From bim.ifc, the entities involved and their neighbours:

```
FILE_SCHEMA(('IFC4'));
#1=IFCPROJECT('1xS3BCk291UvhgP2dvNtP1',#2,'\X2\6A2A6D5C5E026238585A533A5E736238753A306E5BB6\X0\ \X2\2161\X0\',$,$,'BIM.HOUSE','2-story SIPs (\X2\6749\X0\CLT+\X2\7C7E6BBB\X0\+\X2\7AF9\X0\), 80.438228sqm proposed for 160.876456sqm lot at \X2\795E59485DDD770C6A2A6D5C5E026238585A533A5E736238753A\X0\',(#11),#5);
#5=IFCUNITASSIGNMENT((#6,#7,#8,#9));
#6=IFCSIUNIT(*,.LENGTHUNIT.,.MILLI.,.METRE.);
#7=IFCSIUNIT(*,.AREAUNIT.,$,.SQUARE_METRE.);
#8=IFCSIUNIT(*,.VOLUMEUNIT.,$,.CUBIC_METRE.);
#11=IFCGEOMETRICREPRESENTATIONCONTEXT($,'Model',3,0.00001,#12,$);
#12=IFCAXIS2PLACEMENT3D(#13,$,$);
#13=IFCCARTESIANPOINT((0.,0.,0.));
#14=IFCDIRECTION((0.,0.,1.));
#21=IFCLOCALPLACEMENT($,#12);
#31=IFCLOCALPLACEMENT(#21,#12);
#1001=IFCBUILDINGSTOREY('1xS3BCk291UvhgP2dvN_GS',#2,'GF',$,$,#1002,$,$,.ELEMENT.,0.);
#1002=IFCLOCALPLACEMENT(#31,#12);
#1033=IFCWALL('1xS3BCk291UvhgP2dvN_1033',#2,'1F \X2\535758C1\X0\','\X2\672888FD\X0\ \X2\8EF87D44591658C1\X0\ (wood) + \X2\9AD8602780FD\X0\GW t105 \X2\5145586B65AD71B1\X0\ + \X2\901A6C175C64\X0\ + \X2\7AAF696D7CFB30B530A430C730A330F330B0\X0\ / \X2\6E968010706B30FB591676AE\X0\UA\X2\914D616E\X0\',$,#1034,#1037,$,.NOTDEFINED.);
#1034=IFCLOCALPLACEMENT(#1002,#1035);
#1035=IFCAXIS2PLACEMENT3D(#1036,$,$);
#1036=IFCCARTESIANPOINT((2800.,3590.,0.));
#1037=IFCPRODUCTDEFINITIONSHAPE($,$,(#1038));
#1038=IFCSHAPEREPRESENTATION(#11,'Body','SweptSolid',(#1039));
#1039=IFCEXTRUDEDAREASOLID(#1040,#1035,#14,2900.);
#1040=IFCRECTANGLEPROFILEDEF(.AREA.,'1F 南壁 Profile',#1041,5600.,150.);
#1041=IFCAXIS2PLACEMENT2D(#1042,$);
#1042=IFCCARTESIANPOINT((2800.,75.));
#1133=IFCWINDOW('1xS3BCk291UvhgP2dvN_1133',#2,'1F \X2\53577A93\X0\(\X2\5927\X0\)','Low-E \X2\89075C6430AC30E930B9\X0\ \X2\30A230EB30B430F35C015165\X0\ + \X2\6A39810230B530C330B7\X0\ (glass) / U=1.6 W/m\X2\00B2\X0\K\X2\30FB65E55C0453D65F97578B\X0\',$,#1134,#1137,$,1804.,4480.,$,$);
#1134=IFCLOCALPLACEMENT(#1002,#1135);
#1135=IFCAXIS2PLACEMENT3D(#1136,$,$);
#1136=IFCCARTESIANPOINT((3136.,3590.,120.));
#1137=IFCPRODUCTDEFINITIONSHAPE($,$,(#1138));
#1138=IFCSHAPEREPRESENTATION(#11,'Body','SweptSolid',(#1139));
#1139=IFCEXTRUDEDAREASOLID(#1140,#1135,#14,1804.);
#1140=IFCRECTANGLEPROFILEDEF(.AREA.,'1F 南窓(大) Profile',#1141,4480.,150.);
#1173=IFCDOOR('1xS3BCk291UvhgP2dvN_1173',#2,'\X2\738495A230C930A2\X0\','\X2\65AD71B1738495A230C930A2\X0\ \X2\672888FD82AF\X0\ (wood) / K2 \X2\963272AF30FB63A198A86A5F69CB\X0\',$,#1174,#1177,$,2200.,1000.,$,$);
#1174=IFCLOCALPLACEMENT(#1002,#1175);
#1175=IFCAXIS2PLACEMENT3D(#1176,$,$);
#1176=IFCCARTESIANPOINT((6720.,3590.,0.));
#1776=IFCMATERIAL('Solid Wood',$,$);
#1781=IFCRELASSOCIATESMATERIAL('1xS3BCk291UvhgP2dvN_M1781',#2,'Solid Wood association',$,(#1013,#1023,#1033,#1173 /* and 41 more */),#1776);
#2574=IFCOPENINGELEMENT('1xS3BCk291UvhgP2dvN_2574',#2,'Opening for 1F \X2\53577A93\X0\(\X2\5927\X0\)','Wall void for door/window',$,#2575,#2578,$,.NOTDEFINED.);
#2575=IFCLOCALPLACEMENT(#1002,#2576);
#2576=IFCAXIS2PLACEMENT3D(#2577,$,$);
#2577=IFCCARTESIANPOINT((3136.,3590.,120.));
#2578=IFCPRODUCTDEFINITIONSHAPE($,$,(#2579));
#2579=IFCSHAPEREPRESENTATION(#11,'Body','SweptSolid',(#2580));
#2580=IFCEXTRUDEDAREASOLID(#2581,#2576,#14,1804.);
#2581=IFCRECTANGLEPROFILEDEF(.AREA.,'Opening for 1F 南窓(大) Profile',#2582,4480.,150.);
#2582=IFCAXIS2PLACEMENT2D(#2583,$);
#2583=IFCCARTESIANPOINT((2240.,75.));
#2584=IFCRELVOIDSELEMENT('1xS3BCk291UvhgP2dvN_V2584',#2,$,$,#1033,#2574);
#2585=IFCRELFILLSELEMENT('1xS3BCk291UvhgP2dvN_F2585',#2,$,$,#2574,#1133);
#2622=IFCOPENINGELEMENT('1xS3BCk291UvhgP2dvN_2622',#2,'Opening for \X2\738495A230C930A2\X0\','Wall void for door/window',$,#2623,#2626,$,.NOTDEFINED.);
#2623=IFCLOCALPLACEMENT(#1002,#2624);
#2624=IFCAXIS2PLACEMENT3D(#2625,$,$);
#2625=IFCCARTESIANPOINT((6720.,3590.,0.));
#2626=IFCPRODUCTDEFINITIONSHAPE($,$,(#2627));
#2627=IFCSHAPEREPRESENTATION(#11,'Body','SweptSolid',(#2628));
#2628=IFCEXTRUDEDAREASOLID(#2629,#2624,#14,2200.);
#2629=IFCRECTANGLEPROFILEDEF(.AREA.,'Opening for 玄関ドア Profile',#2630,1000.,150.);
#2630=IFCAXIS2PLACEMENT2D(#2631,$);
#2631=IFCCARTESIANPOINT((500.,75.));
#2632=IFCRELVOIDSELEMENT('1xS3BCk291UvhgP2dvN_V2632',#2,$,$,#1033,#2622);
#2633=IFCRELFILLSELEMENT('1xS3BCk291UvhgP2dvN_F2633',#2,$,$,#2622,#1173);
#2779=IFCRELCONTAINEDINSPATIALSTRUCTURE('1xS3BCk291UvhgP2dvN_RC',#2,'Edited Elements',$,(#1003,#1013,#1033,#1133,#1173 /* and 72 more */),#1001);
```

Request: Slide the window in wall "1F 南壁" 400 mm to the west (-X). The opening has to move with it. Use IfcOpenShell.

```python
import ifcopenshell
import ifcopenshell.api.geometry
import ifcopenshell.util.placement

model = ifcopenshell.open("bim.ifc")

window = model.by_guid("1xS3BCk291UvhgP2dvN_1133")
opening = window.FillsVoids[0].RelatingOpeningElement
wall = opening.VoidsElements[0].RelatingBuildingElement

wall_matrix = ifcopenshell.util.placement.get_local_placement(wall.ObjectPlacement)
shift = wall_matrix[:3, 0] * -400.0
before = ifcopenshell.util.placement.get_local_placement(window.ObjectPlacement)[:3, 3].copy()

# The window is not placed relative to its opening, so move both.
for product in (opening, window):
    matrix = ifcopenshell.util.placement.get_local_placement(product.ObjectPlacement)
    matrix[:3, 3] += shift
    ifcopenshell.api.geometry.edit_object_placement(model, product=product, matrix=matrix, is_si=False)

after = ifcopenshell.util.placement.get_local_placement(window.ObjectPlacement)[:3, 3]
print("window moved by", (after - before).round(3) + 0.0)

model.write("bim_updated.ifc")
```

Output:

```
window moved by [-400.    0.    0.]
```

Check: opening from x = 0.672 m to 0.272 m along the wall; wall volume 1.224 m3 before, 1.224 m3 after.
